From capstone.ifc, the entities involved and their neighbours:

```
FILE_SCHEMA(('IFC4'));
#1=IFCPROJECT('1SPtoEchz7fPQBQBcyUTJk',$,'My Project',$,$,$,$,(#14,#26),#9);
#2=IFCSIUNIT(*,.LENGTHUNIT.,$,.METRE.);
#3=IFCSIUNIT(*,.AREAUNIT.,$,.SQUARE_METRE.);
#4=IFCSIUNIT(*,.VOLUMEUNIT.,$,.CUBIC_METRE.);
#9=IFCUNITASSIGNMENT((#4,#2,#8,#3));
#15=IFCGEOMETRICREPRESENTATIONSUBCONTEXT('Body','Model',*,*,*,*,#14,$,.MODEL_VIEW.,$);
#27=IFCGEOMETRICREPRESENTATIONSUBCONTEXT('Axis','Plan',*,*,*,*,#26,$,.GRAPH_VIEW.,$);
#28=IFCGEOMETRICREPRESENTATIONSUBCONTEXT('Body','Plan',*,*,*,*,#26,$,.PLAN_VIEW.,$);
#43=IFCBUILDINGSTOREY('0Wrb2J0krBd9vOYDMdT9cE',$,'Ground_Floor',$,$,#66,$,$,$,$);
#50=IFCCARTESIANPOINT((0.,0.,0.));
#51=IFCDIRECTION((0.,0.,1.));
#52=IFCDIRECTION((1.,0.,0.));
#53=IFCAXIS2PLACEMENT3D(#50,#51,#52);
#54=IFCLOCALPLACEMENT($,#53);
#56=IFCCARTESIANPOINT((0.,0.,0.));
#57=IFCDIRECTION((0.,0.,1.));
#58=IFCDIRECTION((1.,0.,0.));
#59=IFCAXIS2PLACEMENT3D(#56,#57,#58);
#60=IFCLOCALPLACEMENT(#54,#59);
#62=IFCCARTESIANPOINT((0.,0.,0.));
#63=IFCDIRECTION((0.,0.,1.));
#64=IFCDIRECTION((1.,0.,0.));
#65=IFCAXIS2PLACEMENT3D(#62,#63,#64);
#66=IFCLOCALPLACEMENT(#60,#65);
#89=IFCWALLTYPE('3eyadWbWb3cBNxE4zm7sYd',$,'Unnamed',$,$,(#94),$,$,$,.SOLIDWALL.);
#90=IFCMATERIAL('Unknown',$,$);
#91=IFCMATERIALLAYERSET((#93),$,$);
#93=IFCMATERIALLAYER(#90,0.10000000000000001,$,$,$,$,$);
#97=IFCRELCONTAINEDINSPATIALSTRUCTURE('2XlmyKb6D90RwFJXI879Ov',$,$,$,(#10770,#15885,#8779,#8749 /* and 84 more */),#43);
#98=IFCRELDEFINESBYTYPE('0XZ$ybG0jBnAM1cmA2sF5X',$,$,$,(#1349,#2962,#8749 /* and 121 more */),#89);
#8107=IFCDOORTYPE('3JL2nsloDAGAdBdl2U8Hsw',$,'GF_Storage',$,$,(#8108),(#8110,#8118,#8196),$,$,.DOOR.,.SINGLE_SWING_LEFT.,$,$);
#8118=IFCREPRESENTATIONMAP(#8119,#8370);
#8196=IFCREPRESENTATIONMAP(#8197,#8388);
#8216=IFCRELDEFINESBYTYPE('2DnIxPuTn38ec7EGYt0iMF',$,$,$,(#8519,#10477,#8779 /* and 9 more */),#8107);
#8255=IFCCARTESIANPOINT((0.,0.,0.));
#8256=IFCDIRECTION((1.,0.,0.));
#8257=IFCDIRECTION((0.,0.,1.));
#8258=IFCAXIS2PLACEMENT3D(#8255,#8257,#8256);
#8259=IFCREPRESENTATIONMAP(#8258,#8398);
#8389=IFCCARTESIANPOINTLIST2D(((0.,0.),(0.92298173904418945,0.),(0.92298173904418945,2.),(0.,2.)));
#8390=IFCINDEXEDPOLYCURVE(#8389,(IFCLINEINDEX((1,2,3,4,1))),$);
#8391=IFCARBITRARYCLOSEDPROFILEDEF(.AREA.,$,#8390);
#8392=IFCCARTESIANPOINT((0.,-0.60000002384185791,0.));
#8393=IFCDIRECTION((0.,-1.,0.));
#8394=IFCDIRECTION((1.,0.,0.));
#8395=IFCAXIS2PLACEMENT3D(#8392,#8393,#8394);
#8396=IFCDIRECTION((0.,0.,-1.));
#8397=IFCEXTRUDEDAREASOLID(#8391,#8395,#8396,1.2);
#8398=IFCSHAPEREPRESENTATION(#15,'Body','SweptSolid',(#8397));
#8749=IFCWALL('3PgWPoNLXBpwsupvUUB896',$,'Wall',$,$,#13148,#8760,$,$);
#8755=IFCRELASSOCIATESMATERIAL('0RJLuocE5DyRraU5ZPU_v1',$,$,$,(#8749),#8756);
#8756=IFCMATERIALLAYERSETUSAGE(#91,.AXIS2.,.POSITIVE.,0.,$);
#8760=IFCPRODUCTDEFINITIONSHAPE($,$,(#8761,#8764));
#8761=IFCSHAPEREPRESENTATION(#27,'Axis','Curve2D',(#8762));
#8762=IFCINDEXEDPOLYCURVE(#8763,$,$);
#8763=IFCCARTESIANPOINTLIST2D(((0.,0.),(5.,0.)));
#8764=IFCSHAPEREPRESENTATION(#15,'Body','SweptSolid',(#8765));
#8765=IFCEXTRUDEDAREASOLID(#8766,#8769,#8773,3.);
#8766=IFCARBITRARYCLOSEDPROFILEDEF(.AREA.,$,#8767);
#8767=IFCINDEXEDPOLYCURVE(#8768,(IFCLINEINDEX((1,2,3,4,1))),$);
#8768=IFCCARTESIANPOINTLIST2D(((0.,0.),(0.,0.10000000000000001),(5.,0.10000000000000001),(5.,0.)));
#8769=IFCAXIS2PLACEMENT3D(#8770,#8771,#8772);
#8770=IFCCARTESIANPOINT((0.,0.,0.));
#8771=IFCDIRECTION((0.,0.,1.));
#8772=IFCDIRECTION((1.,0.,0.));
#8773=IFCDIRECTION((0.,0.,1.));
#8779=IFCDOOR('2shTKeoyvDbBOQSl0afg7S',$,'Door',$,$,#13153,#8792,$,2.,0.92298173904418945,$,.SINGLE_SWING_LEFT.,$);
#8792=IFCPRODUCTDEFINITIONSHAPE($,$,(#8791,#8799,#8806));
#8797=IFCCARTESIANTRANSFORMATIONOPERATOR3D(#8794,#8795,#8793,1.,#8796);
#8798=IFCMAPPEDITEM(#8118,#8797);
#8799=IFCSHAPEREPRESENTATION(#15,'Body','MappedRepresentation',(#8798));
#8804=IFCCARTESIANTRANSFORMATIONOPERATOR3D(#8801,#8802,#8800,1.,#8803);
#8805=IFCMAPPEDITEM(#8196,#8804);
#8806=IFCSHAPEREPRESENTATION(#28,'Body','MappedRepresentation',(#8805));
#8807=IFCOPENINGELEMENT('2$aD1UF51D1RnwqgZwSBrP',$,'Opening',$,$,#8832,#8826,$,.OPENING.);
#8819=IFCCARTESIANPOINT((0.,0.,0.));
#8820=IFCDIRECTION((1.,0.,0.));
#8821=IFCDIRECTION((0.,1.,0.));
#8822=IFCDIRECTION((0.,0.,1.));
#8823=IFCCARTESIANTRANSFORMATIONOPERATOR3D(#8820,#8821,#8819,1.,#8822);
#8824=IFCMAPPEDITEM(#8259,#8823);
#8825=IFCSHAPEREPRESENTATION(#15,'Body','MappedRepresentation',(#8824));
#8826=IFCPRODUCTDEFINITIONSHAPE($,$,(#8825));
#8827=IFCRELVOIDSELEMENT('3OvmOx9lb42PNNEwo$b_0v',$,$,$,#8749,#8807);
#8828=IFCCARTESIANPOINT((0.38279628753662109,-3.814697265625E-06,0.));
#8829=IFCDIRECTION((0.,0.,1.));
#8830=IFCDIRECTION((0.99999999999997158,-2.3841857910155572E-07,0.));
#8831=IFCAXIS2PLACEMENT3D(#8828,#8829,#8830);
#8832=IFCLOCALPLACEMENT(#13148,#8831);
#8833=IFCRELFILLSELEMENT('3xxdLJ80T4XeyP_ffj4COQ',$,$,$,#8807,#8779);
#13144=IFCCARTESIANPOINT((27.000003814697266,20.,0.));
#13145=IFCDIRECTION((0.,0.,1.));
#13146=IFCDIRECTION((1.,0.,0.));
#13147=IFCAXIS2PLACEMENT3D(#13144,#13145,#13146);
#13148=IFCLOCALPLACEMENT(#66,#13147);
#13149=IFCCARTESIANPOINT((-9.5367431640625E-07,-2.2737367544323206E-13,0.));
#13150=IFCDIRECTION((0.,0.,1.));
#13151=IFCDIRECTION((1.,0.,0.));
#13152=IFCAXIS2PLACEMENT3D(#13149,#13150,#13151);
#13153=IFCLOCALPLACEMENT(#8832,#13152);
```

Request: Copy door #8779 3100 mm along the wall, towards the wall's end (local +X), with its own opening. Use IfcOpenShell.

```python
import ifcopenshell
import ifcopenshell.api.feature
import ifcopenshell.api.geometry
import ifcopenshell.api.root
import ifcopenshell.geom
import ifcopenshell.util.element
import ifcopenshell.util.placement
import ifcopenshell.util.shape
import ifcopenshell.util.unit

model = ifcopenshell.open("capstone.ifc")
unit_scale = ifcopenshell.util.unit.calculate_unit_scale(model)
settings = ifcopenshell.geom.settings()


def volume(element):
    """Net volume in cubic metres, openings subtracted."""
    shape = ifcopenshell.geom.create_shape(settings, element)
    return ifcopenshell.util.shape.get_volume(shape.geometry)


door = model.by_id(8779)
opening = door.FillsVoids[0].RelatingOpeningElement
wall = opening.VoidsElements[0].RelatingBuildingElement
before = volume(wall)
shift = ifcopenshell.util.placement.get_local_placement(wall.ObjectPlacement)[:3, 0] * 3.1 / unit_scale

# copy_class copies the void relationship, type, container and properties, but no geometry.
new_opening = ifcopenshell.api.root.copy_class(model, product=opening)
new_opening.Representation = ifcopenshell.util.element.copy_deep(
    model, opening.Representation, exclude=["IfcGeometricRepresentationContext", "IfcRepresentationMap"]
)
new_door = ifcopenshell.api.root.copy_class(model, product=door)
new_door.Representation = ifcopenshell.util.element.copy_deep(
    model, door.Representation, exclude=["IfcGeometricRepresentationContext", "IfcRepresentationMap"]
)
ifcopenshell.api.feature.add_filling(model, opening=new_opening, element=new_door)

for old, new in ((opening, new_opening), (door, new_door)):
    matrix = ifcopenshell.util.placement.get_local_placement(old.ObjectPlacement)
    matrix[:3, 3] += shift
    ifcopenshell.api.geometry.edit_object_placement(model, product=new, matrix=matrix, is_si=False)

after = volume(wall)

print(f"wall volume {before:.3f} -> {after:.3f} m3")

model.write("capstone_updated.ifc")
```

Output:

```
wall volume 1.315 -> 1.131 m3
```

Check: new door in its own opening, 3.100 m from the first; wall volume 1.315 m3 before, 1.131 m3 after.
